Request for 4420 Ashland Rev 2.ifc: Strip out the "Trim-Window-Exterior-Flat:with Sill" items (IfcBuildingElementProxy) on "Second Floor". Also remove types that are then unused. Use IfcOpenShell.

First a look at what the model holds.

```python
import ifcopenshell
import ifcopenshell.util.element

model = ifcopenshell.open("4420 Ashland Rev 2.ifc")
print(model.schema)
storey = next(s for s in model.by_type("IfcBuildingStorey") if s.Name == "Second Floor")
proxies = [e for e in ifcopenshell.util.element.get_decomposition(storey) if e.is_a("IfcBuildingElementProxy")]
seen = {}
for e in proxies:
    element_type = ifcopenshell.util.element.get_type(e)
    name = element_type.Name if element_type not in (None, e) else None
    seen[name] = seen.get(name, 0) + 1
for name, count in sorted(seen.items(), key=str):
    print(count, "x", name)
```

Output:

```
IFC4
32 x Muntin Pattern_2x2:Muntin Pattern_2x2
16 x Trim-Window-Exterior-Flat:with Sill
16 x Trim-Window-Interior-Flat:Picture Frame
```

```python
import ifcopenshell
import ifcopenshell.api.root
import ifcopenshell.util.element

model = ifcopenshell.open("4420 Ashland Rev 2.ifc")

storey = next(s for s in model.by_type("IfcBuildingStorey") if s.Name == "Second Floor")
proxies = [e for e in ifcopenshell.util.element.get_decomposition(storey) if e.is_a("IfcBuildingElementProxy")]
targets = [e for e in proxies if (t := ifcopenshell.util.element.get_type(e)) not in (None, e) and t.Name == "Trim-Window-Exterior-Flat:with Sill"]
types = {ifcopenshell.util.element.get_type(e) for e in targets} - {None, *targets}

for e in targets:
    ifcopenshell.api.root.remove_product(model, product=e)
print(len(targets), "removed")

unused = [t for t in types if not ifcopenshell.util.element.get_types(t)]
for t in unused:
    ifcopenshell.api.root.remove_product(model, product=t)
print(len(unused), "unused types removed")

model.write("4420 Ashland Rev 2_updated.ifc")
```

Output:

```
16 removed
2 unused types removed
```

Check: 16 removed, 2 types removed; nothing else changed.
